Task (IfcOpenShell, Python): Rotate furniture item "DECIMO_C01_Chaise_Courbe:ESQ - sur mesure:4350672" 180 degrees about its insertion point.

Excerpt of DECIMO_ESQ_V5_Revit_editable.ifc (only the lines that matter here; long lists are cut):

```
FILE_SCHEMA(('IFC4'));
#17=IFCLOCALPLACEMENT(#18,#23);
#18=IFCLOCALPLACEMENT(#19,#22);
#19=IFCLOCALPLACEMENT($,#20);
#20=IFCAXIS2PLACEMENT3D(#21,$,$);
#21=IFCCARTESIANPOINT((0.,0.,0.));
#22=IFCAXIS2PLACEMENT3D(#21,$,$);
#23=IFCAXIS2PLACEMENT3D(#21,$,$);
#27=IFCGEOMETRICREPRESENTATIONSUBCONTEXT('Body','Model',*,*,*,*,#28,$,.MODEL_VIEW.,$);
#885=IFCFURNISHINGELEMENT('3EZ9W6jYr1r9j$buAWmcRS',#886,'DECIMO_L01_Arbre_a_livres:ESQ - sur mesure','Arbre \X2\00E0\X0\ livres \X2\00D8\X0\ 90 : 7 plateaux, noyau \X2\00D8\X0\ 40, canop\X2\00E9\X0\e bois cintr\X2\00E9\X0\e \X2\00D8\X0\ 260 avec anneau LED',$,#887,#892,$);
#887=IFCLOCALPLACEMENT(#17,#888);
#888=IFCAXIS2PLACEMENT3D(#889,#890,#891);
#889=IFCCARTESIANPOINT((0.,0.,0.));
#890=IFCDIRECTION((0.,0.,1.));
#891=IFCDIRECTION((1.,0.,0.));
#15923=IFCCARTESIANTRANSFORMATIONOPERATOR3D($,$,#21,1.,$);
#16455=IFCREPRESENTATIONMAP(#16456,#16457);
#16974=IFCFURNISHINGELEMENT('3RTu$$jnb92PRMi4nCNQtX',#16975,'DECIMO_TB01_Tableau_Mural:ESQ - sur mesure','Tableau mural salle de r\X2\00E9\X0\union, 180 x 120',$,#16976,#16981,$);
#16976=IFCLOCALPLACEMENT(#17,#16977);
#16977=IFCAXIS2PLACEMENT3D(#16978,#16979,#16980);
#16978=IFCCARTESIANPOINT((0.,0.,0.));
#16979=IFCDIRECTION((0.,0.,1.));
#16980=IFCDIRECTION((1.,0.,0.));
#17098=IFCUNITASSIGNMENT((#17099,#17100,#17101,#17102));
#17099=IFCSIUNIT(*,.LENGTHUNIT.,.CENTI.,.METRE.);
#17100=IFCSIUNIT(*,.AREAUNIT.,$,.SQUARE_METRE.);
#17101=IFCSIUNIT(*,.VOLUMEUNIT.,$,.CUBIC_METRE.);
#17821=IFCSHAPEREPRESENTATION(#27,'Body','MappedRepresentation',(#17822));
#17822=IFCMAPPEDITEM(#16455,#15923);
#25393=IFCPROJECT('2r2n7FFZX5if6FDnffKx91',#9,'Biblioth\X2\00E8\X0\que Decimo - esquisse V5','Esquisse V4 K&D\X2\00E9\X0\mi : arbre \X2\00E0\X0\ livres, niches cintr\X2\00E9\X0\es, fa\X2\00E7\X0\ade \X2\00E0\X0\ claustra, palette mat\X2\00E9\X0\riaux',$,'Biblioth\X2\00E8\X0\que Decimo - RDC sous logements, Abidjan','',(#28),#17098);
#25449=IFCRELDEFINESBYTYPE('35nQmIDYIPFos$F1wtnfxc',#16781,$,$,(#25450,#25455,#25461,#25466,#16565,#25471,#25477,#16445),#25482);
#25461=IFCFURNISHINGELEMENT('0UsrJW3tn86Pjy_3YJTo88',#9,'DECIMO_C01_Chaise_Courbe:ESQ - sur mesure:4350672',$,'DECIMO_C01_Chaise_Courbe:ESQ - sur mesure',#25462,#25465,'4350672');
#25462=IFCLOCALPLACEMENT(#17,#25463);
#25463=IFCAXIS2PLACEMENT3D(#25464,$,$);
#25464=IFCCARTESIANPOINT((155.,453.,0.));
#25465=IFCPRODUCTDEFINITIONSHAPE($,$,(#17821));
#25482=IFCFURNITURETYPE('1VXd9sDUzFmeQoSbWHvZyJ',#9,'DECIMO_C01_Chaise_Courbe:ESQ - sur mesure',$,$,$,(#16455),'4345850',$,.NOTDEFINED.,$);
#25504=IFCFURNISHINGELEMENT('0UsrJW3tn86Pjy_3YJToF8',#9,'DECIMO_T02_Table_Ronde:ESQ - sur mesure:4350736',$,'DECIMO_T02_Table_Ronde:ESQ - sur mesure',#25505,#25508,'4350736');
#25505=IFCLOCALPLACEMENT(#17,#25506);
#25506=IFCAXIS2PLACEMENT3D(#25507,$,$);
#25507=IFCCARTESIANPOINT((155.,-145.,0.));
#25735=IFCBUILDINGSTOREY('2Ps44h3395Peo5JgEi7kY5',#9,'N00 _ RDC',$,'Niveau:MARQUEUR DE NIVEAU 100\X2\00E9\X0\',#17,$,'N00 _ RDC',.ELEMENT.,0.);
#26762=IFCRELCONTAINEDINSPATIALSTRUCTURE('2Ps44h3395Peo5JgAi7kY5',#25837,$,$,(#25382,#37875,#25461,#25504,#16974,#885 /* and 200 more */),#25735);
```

```python
import ifcopenshell
import ifcopenshell.api.geometry
import ifcopenshell.util.placement

model = ifcopenshell.open("DECIMO_ESQ_V5_Revit_editable.ifc")

item = model.by_guid("0UsrJW3tn86Pjy_3YJTo88")
matrix = ifcopenshell.util.placement.get_local_placement(item.ObjectPlacement)
matrix = matrix @ ifcopenshell.util.placement.rotation(180, "Z")
ifcopenshell.api.geometry.edit_object_placement(model, product=item, matrix=matrix, is_si=False)

print(ifcopenshell.util.placement.get_local_placement(item.ObjectPlacement).round(3) + 0.0)

model.write("DECIMO_ESQ_V5_Revit_editable-out.ifc")
```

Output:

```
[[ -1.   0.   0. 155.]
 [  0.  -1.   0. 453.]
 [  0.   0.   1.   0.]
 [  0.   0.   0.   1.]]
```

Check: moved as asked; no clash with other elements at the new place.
